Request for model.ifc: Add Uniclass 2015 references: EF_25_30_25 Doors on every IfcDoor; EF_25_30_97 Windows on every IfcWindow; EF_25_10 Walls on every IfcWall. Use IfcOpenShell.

First a look at what the model holds.

```python
import ifcopenshell

model = ifcopenshell.open("model.ifc")
print(model.schema)
print("classifications:", [c.Name for c in model.by_type("IfcClassification")])
for ifc_class in ("IfcDoor", "IfcRoof", "IfcStair", "IfcWall", "IfcWindow"):
    print(ifc_class, len(model.by_type(ifc_class)))
```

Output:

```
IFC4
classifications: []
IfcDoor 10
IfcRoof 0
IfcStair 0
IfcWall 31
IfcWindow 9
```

```python
import ifcopenshell
import ifcopenshell.api.classification

model = ifcopenshell.open("model.ifc")

system = ifcopenshell.api.classification.add_classification(model, classification="Uniclass 2015")

codes = {
    "IfcDoor": ("EF_25_30_25", "Doors"),
    "IfcWindow": ("EF_25_30_97", "Windows"),
    "IfcWall": ("EF_25_10", "Walls"),
}
for ifc_class, (code, name) in codes.items():
    products = model.by_type(ifc_class)
    ifcopenshell.api.classification.add_reference(
        model, products=products, classification=system, identification=code, name=name
    )
    print(code, len(products))

model.write("model-out.ifc")
```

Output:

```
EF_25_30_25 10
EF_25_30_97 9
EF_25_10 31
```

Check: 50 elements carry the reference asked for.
